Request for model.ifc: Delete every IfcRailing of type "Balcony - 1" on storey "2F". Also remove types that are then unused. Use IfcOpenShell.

First a look at what the model holds.

```python
import ifcopenshell
import ifcopenshell.util.element

model = ifcopenshell.open("model.ifc")
print(model.schema)
storey = next(s for s in model.by_type("IfcBuildingStorey") if s.Name == "2F")
railings = [e for e in ifcopenshell.util.element.get_decomposition(storey) if e.is_a("IfcRailing")]
seen = {}
for e in railings:
    element_type = ifcopenshell.util.element.get_type(e)
    name = element_type.Name if element_type not in (None, e) else None
    seen[name] = seen.get(name, 0) + 1
for name, count in sorted(seen.items(), key=str):
    print(count, "x", name)
```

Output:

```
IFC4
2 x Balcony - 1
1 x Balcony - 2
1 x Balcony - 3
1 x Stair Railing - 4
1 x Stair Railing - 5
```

```python
import ifcopenshell
import ifcopenshell.api.root
import ifcopenshell.util.element

model = ifcopenshell.open("model.ifc")

storey = next(s for s in model.by_type("IfcBuildingStorey") if s.Name == "2F")
railings = [e for e in ifcopenshell.util.element.get_decomposition(storey) if e.is_a("IfcRailing")]
targets = [e for e in railings if (t := ifcopenshell.util.element.get_type(e)) not in (None, e) and t.Name == "Balcony - 1"]
types = {ifcopenshell.util.element.get_type(e) for e in targets} - {None, *targets}

for e in targets:
    ifcopenshell.api.root.remove_product(model, product=e)
print(len(targets), "removed")

unused = [t for t in types if not ifcopenshell.util.element.get_types(t)]
for t in unused:
    ifcopenshell.api.root.remove_product(model, product=t)
print(len(unused), "unused types removed")

model.write("model-out.ifc")
```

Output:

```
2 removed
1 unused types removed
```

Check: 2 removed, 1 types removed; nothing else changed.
